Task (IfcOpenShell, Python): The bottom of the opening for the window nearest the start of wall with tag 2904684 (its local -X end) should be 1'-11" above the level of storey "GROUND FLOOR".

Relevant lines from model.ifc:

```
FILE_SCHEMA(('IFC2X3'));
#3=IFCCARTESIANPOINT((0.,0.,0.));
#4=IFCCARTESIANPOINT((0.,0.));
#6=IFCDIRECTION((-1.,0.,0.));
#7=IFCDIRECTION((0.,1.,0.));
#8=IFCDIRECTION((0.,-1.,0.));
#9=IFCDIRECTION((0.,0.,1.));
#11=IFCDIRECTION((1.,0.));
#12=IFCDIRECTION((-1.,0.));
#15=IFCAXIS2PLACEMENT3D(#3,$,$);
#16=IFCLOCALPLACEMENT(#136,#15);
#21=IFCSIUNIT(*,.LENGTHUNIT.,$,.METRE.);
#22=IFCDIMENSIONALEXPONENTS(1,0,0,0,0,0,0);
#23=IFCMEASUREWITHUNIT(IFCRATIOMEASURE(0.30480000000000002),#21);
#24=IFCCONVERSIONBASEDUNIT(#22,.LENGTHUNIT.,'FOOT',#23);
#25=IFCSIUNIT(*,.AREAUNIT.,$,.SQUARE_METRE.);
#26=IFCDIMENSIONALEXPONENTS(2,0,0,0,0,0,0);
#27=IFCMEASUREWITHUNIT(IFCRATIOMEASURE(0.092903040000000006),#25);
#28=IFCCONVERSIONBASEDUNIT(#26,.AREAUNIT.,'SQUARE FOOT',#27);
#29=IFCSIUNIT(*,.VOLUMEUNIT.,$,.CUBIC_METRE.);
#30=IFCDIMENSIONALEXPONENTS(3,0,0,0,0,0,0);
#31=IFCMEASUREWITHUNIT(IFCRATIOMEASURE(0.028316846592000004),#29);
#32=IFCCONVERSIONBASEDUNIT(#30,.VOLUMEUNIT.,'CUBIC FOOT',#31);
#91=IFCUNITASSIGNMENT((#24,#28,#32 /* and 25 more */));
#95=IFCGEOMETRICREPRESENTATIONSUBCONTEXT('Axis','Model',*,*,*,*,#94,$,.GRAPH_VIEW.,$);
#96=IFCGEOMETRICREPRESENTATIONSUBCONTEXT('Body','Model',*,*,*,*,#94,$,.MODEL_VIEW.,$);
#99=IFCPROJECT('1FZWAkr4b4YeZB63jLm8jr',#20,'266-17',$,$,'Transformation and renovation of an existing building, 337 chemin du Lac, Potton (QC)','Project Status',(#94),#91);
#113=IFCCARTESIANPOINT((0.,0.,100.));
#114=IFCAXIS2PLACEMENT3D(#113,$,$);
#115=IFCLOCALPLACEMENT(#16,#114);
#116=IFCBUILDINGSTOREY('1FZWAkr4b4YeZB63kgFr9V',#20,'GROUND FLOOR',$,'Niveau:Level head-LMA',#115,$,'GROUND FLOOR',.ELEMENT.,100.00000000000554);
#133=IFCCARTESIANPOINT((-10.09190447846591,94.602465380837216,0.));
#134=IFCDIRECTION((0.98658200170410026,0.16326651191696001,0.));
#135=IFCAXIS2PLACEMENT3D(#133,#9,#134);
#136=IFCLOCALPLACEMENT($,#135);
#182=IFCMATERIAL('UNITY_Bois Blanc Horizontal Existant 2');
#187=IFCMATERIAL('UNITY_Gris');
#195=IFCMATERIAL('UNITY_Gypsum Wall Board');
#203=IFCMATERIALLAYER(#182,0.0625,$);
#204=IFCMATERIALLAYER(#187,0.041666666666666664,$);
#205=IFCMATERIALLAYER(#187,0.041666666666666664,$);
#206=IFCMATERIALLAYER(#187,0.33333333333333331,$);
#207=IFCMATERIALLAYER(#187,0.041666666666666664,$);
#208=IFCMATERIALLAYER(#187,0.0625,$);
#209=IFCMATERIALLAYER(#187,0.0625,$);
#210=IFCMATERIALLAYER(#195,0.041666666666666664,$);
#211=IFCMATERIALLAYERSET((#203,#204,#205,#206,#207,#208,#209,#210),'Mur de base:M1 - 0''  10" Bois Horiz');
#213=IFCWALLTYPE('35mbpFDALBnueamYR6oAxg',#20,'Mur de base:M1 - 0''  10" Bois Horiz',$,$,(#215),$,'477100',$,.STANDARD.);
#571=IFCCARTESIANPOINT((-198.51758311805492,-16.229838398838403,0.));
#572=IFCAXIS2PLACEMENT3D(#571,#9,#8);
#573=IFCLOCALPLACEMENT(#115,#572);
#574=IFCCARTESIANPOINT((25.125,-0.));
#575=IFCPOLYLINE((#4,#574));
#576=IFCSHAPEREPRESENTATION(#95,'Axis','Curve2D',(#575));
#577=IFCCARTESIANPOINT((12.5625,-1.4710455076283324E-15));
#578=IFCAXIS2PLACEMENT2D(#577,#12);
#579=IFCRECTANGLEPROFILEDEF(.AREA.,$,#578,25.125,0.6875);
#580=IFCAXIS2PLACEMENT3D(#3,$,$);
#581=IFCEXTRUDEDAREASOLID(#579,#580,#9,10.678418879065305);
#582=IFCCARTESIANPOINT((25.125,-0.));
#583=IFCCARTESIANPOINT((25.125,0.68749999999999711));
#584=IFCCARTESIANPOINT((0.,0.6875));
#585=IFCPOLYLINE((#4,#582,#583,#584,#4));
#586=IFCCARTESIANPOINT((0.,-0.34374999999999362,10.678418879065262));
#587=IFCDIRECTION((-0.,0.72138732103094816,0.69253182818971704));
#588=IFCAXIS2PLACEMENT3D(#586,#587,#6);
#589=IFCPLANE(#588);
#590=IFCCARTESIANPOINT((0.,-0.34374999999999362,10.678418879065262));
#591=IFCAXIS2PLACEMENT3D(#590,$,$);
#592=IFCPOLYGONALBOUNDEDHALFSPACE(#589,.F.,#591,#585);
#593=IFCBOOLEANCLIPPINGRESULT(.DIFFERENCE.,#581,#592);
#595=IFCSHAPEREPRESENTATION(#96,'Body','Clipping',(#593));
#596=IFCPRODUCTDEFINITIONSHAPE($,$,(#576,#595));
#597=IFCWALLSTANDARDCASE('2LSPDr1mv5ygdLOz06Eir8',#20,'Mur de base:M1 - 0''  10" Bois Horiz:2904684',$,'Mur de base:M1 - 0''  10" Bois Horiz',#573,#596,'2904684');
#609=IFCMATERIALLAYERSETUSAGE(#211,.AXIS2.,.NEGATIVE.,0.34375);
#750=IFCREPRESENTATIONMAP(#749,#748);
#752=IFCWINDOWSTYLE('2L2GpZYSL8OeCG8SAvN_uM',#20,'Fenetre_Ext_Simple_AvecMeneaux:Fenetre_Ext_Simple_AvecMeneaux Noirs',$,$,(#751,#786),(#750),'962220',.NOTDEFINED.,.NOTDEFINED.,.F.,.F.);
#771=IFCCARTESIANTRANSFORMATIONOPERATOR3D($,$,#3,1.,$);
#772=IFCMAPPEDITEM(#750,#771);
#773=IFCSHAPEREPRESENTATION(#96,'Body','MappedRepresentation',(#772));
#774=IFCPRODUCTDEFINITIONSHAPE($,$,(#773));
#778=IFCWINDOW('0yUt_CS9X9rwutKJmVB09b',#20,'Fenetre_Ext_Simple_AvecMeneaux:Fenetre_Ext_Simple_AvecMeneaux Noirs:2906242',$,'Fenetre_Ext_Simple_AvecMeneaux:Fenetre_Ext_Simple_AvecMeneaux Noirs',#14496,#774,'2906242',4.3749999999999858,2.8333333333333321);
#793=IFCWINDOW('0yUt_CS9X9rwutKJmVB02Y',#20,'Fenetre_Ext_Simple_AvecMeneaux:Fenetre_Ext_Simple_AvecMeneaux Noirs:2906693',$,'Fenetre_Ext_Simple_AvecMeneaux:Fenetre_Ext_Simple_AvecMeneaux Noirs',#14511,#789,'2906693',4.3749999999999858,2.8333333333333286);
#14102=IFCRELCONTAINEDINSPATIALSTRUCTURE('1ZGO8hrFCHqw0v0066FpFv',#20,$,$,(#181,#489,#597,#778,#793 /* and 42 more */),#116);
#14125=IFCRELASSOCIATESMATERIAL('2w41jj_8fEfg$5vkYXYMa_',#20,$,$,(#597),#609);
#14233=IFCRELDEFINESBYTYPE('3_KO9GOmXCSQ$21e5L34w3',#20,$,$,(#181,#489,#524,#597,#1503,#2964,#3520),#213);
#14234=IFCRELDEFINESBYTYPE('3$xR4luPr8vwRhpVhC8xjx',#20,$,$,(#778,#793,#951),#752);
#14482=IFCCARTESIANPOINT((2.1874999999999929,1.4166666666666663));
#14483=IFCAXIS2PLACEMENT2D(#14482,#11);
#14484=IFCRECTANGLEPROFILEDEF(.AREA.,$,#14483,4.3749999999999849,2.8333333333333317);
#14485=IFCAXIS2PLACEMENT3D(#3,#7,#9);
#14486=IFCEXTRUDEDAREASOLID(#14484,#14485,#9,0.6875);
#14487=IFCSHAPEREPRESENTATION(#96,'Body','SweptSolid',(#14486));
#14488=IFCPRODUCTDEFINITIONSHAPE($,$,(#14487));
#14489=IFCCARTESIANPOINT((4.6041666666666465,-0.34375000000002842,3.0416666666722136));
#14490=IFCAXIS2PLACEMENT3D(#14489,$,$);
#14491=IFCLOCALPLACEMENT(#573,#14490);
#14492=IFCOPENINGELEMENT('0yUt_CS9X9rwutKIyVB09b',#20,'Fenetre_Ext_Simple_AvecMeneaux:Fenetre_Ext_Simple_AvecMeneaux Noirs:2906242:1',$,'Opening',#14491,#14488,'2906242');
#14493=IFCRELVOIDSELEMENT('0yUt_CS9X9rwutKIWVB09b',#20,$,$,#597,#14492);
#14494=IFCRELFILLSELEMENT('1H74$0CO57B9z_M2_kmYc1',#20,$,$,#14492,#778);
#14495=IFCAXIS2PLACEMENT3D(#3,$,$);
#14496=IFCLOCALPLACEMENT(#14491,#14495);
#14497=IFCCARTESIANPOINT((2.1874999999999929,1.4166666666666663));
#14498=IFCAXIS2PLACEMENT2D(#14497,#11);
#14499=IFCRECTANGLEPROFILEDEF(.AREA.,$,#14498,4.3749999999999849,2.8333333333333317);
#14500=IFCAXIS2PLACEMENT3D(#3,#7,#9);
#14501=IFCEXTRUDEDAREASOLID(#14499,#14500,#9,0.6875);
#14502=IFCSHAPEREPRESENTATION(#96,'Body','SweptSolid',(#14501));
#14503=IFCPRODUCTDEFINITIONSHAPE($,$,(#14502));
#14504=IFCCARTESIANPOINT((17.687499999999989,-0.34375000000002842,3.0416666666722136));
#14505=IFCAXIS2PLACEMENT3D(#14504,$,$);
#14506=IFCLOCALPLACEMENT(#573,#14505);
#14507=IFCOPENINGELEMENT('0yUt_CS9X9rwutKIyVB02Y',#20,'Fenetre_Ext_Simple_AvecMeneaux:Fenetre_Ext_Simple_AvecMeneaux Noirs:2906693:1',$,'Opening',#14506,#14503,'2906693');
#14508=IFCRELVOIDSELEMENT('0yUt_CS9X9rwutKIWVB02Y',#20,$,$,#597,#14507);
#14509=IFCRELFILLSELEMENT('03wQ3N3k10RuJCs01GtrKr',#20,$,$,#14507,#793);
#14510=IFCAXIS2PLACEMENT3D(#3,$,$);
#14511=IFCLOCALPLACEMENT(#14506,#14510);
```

```python
import numpy as np
import ifcopenshell
import ifcopenshell.api.geometry
import ifcopenshell.geom
import ifcopenshell.util.element
import ifcopenshell.util.placement
import ifcopenshell.util.shape
import ifcopenshell.util.unit

model = ifcopenshell.open("model.ifc")
unit_scale = ifcopenshell.util.unit.calculate_unit_scale(model)

window = model.by_id(778)
opening = window.FillsVoids[0].RelatingOpeningElement
storey = ifcopenshell.util.element.get_container(window, ifc_class="IfcBuildingStorey")
level = ifcopenshell.util.placement.get_local_placement(storey.ObjectPlacement)[2, 3]

# The opening's origin need not be at the sill, so measure its lowest point.
shape = ifcopenshell.geom.create_shape(ifcopenshell.geom.settings(), opening)
bottom = ifcopenshell.util.shape.get_shape_bottom_elevation(shape, shape.geometry) / unit_scale
dz = level + 23 * 0.0254 / unit_scale - bottom

shift = np.array([0.0, 0.0, dz])
# The window is placed relative to its opening, so it follows when the opening moves.
matrix = ifcopenshell.util.placement.get_local_placement(opening.ObjectPlacement)
matrix[:3, 3] += shift
ifcopenshell.api.geometry.edit_object_placement(
    model, product=opening, matrix=matrix, is_si=False, should_transform_children=True
)

print(f"moved by {dz * unit_scale:+.3f} m")

model.write("model_rev.ifc")
```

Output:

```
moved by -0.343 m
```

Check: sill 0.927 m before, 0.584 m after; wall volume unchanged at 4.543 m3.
